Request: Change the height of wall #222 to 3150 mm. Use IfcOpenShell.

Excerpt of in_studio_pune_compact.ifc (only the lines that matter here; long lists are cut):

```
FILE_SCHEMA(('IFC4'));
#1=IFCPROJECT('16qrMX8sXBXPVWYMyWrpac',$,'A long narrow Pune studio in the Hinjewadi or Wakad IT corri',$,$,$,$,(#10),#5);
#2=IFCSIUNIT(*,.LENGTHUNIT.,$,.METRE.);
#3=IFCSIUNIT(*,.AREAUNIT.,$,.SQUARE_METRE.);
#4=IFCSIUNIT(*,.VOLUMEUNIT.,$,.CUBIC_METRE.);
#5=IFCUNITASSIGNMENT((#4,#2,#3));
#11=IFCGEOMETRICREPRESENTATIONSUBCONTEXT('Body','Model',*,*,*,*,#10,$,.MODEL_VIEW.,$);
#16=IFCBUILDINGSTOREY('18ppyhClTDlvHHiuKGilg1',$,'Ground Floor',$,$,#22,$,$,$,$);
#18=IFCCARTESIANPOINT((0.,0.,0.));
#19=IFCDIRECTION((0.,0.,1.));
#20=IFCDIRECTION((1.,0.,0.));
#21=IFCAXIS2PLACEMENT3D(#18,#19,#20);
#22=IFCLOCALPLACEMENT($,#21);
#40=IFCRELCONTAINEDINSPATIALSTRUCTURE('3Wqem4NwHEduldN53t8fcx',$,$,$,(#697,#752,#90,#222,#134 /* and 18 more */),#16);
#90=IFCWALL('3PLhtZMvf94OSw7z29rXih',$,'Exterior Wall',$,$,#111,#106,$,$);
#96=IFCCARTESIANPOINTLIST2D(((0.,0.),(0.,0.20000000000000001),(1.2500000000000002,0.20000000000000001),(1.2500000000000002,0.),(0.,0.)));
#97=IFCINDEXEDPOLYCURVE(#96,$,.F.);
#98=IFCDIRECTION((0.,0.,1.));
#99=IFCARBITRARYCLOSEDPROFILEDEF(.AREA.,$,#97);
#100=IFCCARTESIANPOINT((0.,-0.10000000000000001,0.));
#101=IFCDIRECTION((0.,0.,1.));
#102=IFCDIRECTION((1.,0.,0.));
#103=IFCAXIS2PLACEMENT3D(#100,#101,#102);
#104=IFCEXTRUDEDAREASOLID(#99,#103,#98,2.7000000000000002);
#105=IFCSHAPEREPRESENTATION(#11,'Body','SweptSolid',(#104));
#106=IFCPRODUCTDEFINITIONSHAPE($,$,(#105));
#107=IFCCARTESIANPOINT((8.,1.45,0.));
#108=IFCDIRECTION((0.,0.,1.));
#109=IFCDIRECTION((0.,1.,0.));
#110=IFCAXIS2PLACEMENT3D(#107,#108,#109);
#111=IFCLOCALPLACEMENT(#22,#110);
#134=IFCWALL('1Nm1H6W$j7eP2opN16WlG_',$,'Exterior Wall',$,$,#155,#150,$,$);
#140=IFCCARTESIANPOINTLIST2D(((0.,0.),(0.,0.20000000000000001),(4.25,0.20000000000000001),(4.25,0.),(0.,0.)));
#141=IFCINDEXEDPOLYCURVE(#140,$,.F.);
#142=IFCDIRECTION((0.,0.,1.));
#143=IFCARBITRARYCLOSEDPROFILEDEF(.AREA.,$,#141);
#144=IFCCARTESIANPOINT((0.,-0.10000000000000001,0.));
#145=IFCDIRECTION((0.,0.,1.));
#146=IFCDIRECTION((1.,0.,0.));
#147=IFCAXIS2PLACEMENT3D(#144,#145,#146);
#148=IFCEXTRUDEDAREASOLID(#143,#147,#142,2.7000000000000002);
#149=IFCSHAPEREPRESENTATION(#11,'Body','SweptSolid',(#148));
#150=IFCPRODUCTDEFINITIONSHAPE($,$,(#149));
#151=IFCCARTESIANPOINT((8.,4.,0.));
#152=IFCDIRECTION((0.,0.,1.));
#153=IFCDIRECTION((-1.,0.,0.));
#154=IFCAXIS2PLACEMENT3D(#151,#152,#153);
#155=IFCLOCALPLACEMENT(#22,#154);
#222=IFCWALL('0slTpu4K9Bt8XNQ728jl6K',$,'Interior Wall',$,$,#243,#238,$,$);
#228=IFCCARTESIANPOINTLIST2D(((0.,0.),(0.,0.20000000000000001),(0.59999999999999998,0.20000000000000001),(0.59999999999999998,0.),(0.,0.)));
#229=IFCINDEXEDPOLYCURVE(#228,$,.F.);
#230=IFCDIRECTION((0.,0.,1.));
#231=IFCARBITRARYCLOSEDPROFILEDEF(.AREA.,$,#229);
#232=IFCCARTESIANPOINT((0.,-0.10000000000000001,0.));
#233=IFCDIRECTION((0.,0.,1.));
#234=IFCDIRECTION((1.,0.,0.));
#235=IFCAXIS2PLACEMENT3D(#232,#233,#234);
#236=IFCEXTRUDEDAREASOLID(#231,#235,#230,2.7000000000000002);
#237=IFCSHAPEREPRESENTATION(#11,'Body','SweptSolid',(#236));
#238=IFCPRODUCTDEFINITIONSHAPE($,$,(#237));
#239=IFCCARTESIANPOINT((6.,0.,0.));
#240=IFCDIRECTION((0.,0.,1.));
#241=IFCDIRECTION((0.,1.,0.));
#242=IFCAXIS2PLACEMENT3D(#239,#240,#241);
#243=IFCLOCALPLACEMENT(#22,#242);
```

```python
import ifcopenshell
import ifcopenshell.geom
import ifcopenshell.util.representation
import ifcopenshell.util.shape
import ifcopenshell.util.unit

model = ifcopenshell.open("in_studio_pune_compact.ifc")
unit_scale = ifcopenshell.util.unit.calculate_unit_scale(model)
settings = ifcopenshell.geom.settings()


def volume(element):
    """Net volume in cubic metres, openings subtracted."""
    shape = ifcopenshell.geom.create_shape(settings, element)
    return ifcopenshell.util.shape.get_volume(shape.geometry)


wall = model.by_id(222)
before = volume(wall)

body = ifcopenshell.util.representation.get_representation(wall, "Model", "Body")
solid = body.Items[0]
old_height = solid.Depth
solid.Depth = 3.15 / unit_scale
after = volume(wall)

print(f"height {old_height:g} -> {solid.Depth:g}, volume {before:.3f} -> {after:.3f} m3")

model.write("in_studio_pune_compact_updated.ifc")
```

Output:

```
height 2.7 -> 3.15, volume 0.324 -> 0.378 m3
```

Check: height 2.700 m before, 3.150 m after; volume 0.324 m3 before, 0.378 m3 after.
